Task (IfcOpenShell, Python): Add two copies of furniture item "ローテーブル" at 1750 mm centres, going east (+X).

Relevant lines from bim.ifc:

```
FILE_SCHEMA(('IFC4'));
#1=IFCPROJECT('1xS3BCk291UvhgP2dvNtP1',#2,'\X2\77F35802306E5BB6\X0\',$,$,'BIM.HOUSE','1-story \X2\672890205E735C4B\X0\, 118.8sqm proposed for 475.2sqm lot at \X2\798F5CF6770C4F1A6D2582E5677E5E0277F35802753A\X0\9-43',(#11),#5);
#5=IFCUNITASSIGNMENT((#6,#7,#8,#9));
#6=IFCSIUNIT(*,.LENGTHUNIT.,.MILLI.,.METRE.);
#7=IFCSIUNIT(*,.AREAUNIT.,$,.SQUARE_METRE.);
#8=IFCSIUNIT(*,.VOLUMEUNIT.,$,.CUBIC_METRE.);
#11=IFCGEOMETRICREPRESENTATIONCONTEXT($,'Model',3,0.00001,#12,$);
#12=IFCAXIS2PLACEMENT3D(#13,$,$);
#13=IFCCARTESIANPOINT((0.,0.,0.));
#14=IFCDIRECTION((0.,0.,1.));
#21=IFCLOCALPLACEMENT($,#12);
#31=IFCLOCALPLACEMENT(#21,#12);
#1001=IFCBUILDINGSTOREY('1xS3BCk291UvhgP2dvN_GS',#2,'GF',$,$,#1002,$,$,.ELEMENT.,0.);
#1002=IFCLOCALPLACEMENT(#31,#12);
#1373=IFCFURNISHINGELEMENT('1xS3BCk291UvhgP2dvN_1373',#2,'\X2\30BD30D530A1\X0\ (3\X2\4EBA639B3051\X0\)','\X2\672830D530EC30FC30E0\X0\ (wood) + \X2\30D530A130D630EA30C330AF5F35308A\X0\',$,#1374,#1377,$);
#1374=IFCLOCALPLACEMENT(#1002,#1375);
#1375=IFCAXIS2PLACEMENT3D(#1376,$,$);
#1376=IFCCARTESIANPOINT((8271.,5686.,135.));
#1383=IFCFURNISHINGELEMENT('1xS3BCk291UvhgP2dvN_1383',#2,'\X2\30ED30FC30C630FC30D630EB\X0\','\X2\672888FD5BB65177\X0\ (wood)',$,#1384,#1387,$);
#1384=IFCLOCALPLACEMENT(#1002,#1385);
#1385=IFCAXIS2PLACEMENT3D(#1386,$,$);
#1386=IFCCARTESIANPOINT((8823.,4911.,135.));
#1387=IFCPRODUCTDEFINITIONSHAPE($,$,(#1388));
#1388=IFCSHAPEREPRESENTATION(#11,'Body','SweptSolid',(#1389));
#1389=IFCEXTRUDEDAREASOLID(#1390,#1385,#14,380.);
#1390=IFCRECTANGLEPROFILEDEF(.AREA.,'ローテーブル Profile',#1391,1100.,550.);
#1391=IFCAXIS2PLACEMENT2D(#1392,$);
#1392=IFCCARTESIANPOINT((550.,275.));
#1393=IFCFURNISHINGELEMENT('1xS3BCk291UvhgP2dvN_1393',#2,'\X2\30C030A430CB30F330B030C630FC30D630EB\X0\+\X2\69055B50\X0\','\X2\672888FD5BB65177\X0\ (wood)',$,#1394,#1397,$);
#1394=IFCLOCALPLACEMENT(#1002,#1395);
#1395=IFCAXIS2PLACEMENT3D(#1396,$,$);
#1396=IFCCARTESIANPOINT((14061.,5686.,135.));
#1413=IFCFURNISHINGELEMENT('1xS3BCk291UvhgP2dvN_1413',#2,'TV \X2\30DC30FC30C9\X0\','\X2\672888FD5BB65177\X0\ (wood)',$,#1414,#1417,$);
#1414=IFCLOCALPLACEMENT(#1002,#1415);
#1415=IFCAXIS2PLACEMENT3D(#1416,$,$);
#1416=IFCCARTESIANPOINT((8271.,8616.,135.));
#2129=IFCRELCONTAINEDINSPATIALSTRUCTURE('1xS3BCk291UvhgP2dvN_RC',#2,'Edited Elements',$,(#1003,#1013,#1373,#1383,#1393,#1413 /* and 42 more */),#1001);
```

```python
import numpy as np
import ifcopenshell
import ifcopenshell.api.geometry
import ifcopenshell.api.root
import ifcopenshell.util.element
import ifcopenshell.util.placement
import ifcopenshell.util.unit

model = ifcopenshell.open("bim.ifc")
unit_scale = ifcopenshell.util.unit.calculate_unit_scale(model)


def reuse_history(source, copy):
    """copy_class also copies each property set's owner history, people and application; keep the originals."""
    for rel in copy.IsDefinedBy:
        if rel.is_a("IfcRelDefinesByProperties") and (history := rel.RelatingPropertyDefinition.OwnerHistory):
            rel.RelatingPropertyDefinition.OwnerHistory = source.OwnerHistory
            ifcopenshell.util.element.remove_deep2(model, history)


source = model.by_guid("1xS3BCk291UvhgP2dvN_1383")
base = ifcopenshell.util.placement.get_local_placement(source.ObjectPlacement)
step = np.array([1.0, 0.0, 0.0]) * 1.75 / unit_scale

for i in range(1, 3):
    copy = ifcopenshell.api.root.copy_class(model, product=source)
    copy.Representation = ifcopenshell.util.element.copy_deep(
        model, source.Representation, exclude=["IfcGeometricRepresentationContext", "IfcRepresentationMap"]
    )
    reuse_history(source, copy)
    matrix = base.copy()
    matrix[:3, 3] += i * step
    print("added at", matrix[:3, 3].round(3) + 0.0)
    ifcopenshell.api.geometry.edit_object_placement(model, product=copy, matrix=matrix, is_si=False)

model.write("bim-out.ifc")
```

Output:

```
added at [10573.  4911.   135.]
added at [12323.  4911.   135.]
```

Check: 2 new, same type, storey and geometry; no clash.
